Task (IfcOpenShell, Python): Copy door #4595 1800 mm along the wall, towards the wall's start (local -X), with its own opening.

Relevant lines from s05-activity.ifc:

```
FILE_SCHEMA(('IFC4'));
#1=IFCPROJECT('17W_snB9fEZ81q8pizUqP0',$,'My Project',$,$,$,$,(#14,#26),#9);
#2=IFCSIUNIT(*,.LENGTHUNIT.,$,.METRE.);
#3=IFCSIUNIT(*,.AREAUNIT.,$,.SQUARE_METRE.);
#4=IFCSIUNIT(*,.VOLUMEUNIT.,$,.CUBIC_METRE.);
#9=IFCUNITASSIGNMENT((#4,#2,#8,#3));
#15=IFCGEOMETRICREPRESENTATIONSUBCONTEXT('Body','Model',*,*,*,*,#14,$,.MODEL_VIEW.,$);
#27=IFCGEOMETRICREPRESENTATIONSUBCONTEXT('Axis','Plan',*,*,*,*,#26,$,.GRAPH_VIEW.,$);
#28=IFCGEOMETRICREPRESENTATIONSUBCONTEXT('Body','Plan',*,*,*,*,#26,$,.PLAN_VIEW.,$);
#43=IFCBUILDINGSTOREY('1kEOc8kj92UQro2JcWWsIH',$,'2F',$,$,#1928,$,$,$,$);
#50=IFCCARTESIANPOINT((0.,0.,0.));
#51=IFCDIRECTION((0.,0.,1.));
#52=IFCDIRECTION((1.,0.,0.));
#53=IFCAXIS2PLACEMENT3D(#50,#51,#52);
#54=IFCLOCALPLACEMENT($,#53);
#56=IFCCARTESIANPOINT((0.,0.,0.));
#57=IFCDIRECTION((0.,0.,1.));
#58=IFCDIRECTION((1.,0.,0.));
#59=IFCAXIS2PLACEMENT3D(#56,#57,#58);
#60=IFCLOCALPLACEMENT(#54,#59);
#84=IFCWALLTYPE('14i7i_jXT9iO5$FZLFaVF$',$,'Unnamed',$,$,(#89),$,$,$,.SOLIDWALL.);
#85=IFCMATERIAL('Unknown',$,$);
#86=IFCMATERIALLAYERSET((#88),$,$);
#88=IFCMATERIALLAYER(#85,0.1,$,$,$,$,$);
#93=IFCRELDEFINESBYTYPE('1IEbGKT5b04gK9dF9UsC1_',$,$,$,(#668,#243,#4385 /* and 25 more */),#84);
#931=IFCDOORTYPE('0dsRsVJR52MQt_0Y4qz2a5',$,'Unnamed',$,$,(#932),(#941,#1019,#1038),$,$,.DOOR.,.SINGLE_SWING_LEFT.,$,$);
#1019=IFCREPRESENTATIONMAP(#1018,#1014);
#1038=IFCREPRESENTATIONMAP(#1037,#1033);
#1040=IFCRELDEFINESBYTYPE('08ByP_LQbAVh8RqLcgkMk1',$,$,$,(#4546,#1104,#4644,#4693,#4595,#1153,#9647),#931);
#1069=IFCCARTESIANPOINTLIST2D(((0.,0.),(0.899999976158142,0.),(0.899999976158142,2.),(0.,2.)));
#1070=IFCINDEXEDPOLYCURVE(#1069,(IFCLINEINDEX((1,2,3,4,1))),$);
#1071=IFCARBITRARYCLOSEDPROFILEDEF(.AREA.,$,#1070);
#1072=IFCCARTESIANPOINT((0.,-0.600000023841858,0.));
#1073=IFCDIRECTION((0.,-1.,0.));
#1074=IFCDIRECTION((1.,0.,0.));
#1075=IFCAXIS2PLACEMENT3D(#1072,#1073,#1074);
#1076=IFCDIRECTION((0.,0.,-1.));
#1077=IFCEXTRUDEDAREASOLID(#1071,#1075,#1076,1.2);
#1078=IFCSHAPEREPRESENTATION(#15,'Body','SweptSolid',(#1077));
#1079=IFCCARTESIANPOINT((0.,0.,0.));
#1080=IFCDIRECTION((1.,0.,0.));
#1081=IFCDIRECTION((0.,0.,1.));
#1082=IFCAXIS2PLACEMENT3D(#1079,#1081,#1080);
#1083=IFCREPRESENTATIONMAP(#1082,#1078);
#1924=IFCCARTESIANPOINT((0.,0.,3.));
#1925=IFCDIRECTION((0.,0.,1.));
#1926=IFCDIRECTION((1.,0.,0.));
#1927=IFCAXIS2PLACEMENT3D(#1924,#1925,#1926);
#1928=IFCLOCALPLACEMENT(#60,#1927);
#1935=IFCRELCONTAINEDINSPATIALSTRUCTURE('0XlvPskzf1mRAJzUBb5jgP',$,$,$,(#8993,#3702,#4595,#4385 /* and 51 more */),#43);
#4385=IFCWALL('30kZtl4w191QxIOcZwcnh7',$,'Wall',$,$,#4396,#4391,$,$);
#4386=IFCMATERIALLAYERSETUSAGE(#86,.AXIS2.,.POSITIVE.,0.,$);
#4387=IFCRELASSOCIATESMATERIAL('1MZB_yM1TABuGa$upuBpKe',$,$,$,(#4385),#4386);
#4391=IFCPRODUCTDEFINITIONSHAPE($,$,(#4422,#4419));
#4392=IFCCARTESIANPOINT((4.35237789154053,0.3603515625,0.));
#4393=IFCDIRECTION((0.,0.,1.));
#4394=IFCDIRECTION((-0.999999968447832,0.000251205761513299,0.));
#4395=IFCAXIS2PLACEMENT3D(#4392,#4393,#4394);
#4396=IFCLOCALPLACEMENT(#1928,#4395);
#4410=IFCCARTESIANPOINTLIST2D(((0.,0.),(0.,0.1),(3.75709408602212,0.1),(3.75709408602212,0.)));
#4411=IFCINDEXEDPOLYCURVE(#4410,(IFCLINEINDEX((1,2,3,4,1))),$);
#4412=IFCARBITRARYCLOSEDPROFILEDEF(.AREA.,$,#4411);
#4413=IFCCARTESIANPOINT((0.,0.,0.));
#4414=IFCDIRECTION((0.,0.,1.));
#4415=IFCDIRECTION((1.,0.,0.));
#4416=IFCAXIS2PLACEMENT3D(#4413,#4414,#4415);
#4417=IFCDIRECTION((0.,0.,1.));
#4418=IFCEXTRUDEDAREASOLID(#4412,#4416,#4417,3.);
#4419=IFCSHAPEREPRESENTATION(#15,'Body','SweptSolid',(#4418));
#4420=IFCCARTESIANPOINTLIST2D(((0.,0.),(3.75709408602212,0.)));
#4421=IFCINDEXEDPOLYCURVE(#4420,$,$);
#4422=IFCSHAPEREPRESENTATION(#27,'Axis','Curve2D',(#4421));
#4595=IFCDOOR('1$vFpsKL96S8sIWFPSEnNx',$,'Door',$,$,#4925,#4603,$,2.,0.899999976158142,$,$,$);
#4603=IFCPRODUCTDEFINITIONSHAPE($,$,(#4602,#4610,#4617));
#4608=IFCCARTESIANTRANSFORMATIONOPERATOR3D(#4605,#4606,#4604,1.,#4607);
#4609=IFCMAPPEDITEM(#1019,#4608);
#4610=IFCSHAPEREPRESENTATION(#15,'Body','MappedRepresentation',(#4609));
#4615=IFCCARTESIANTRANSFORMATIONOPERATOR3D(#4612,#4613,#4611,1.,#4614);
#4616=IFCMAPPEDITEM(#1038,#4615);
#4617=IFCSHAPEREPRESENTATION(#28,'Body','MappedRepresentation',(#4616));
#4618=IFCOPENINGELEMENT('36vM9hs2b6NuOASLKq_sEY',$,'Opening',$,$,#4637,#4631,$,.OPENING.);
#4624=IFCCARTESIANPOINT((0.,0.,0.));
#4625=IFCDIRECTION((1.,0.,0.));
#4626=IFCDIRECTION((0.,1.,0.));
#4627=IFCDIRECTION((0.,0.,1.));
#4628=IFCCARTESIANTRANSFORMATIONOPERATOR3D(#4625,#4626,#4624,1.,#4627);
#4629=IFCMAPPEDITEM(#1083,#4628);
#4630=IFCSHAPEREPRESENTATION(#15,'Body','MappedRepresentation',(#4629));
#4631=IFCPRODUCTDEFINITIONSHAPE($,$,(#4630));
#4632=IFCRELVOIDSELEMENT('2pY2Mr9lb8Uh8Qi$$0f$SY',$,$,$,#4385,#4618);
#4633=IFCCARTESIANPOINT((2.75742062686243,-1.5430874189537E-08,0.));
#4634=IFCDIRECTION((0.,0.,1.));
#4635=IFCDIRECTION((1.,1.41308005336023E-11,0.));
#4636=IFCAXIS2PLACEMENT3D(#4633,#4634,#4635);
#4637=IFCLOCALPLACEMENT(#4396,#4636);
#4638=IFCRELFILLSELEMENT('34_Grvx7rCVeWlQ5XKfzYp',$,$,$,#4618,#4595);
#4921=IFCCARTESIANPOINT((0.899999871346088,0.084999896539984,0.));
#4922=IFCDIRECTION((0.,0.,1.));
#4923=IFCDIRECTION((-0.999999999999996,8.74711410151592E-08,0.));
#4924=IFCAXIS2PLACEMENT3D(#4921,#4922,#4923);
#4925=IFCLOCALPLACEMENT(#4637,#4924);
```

```python
import ifcopenshell
import ifcopenshell.api.feature
import ifcopenshell.api.geometry
import ifcopenshell.api.root
import ifcopenshell.geom
import ifcopenshell.util.element
import ifcopenshell.util.placement
import ifcopenshell.util.shape
import ifcopenshell.util.unit

model = ifcopenshell.open("s05-activity.ifc")
unit_scale = ifcopenshell.util.unit.calculate_unit_scale(model)
settings = ifcopenshell.geom.settings()


def volume(element):
    """Net volume in cubic metres, openings subtracted."""
    shape = ifcopenshell.geom.create_shape(settings, element)
    return ifcopenshell.util.shape.get_volume(shape.geometry)


door = model.by_guid("1$vFpsKL96S8sIWFPSEnNx")
opening = door.FillsVoids[0].RelatingOpeningElement
wall = opening.VoidsElements[0].RelatingBuildingElement
before = volume(wall)
shift = ifcopenshell.util.placement.get_local_placement(wall.ObjectPlacement)[:3, 0] * -1.8 / unit_scale

# copy_class copies the void relationship, type, container and properties, but no geometry.
new_opening = ifcopenshell.api.root.copy_class(model, product=opening)
new_opening.Representation = ifcopenshell.util.element.copy_deep(
    model, opening.Representation, exclude=["IfcGeometricRepresentationContext", "IfcRepresentationMap"]
)
new_door = ifcopenshell.api.root.copy_class(model, product=door)
new_door.Representation = ifcopenshell.util.element.copy_deep(
    model, door.Representation, exclude=["IfcGeometricRepresentationContext", "IfcRepresentationMap"]
)
ifcopenshell.api.feature.add_filling(model, opening=new_opening, element=new_door)

for old, new in ((opening, new_opening), (door, new_door)):
    matrix = ifcopenshell.util.placement.get_local_placement(old.ObjectPlacement)
    matrix[:3, 3] += shift
    ifcopenshell.api.geometry.edit_object_placement(model, product=new, matrix=matrix, is_si=False)

after = volume(wall)

print(f"wall volume {before:.3f} -> {after:.3f} m3")

model.write("s05-activity-out.ifc")
```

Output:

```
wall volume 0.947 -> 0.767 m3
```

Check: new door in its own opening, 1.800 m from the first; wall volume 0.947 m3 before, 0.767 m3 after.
